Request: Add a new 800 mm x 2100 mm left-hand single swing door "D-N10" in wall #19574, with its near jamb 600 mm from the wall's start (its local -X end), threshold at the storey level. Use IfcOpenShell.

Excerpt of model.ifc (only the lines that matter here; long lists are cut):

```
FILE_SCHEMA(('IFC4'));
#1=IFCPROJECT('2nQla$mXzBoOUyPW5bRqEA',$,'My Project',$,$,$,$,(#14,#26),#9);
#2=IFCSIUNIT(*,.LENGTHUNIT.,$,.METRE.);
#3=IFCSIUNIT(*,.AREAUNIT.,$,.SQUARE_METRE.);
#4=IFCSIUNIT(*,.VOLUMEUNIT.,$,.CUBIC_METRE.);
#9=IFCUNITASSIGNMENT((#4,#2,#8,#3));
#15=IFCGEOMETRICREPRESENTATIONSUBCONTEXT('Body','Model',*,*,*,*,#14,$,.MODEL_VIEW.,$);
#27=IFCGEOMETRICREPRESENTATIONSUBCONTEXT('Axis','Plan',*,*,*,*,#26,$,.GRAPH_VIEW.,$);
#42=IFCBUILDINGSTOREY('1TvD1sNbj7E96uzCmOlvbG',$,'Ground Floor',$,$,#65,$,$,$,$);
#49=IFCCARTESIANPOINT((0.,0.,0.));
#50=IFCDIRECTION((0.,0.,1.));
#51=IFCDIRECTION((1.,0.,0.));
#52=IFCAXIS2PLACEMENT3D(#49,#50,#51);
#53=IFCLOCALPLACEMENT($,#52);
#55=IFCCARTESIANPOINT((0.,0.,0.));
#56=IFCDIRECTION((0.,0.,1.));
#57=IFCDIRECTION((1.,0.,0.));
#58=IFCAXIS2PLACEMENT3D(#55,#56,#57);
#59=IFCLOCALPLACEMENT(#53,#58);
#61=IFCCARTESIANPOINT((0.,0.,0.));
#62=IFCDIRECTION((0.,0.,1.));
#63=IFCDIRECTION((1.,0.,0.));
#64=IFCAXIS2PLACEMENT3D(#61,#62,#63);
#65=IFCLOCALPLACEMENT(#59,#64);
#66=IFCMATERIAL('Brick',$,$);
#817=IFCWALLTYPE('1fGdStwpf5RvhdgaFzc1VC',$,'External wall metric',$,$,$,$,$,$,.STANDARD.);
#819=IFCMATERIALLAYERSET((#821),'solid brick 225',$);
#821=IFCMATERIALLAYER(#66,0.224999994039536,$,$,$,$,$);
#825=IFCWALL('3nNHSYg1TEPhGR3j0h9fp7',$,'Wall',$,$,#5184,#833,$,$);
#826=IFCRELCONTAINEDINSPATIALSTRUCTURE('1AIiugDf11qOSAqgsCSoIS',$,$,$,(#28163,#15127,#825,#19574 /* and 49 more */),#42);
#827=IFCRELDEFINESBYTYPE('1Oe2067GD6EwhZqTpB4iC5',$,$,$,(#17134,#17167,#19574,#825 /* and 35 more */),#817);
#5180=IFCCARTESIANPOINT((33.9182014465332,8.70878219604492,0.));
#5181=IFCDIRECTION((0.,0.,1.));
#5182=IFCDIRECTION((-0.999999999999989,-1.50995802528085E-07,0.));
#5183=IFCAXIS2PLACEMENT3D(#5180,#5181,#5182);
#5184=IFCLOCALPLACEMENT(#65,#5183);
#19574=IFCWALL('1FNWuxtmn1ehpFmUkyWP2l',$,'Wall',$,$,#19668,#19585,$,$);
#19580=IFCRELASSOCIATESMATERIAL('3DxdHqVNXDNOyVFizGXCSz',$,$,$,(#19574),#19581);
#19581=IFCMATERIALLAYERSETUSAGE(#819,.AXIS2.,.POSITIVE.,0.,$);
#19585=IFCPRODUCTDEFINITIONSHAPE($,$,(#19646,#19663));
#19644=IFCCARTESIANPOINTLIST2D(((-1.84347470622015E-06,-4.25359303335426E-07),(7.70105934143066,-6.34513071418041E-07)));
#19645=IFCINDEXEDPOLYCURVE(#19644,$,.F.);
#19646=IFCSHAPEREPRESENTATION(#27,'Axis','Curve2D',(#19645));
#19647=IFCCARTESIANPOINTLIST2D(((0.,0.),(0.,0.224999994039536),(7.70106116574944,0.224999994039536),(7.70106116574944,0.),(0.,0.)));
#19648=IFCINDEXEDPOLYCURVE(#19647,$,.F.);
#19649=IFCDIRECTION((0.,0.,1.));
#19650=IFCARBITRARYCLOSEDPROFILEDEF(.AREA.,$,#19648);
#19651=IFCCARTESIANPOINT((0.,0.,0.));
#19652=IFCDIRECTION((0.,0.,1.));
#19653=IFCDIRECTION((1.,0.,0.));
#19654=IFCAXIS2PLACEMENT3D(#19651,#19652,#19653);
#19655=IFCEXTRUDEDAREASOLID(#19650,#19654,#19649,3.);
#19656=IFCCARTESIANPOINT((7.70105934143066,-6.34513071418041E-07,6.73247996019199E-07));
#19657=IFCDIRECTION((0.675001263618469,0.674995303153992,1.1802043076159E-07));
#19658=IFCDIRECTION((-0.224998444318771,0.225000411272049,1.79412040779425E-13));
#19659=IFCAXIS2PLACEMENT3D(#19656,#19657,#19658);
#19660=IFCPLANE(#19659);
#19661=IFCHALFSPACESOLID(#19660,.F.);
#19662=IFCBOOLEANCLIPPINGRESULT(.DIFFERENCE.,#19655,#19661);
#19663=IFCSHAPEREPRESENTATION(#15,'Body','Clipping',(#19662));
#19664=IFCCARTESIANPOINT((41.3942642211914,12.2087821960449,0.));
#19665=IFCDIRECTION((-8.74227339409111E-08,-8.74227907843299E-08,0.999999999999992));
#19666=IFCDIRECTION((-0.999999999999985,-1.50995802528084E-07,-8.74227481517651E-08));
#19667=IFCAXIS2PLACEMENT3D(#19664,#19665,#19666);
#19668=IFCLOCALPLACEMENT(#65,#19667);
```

```python
import numpy as np
import ifcopenshell
import ifcopenshell.api.feature
import ifcopenshell.api.geometry
import ifcopenshell.api.root
import ifcopenshell.api.spatial
import ifcopenshell.geom
import ifcopenshell.util.element
import ifcopenshell.util.placement
import ifcopenshell.util.representation
import ifcopenshell.util.shape
import ifcopenshell.util.unit

model = ifcopenshell.open("model.ifc")
unit_scale = ifcopenshell.util.unit.calculate_unit_scale(model)
settings = ifcopenshell.geom.settings()


def volume(element):
    """Net volume in cubic metres, openings subtracted."""
    shape = ifcopenshell.geom.create_shape(settings, element)
    return ifcopenshell.util.shape.get_volume(shape.geometry)


wall = model.by_id(19574)
storey = ifcopenshell.util.element.get_container(wall, ifc_class="IfcBuildingStorey")
context = ifcopenshell.util.representation.get_context(model, "Model", "Body", "MODEL_VIEW")
before = volume(wall)

width, height, from_end, sill = 0.8, 2.1, 0.6, 0.0  # metres

# The wall runs along its own X axis, and the end named is its -X end.
wall_shape = ifcopenshell.geom.create_shape(settings, wall)
x, y, z = ifcopenshell.util.shape.get_vertices(wall_shape.geometry).T
start = x.min() + from_end
face, thickness = float(y.min()), float(y.max() - y.min())
wall_matrix = ifcopenshell.util.placement.get_local_placement(wall.ObjectPlacement)
level = ifcopenshell.util.placement.get_local_placement(storey.ObjectPlacement)[2, 3]


def in_wall(x, y):
    """Placement at x, y metres in the wall's axes, at sill height."""
    matrix = wall_matrix.copy()
    matrix[:, 3] = wall_matrix @ np.array([x / unit_scale, y / unit_scale, 0.0, 1.0])
    matrix[2, 3] = level + sill / unit_scale
    return matrix


# Opening: a box that overshoots both wall faces by 50 mm.
opening = ifcopenshell.api.root.create_entity(model, ifc_class="IfcOpeningElement", predefined_type="OPENING")
box = ifcopenshell.api.geometry.add_wall_representation(
    model, context=context, length=width, height=height, thickness=thickness + 0.1
)
ifcopenshell.api.geometry.assign_representation(model, product=opening, representation=box)
ifcopenshell.api.geometry.edit_object_placement(model, product=opening, matrix=in_wall(start, face - 0.05), is_si=False)
ifcopenshell.api.feature.add_feature(model, feature=opening, element=wall)

door = ifcopenshell.api.root.create_entity(model, ifc_class="IfcDoor", name="D-N10", predefined_type="DOOR")
door.OverallWidth, door.OverallHeight = width / unit_scale, height / unit_scale
door.OperationType = "SINGLE_SWING_LEFT"
body = ifcopenshell.api.geometry.add_door_representation(
    model,
    context=context,
    overall_width=door.OverallWidth,
    overall_height=door.OverallHeight,
    operation_type="SINGLE_SWING_LEFT",
    lining_properties={"LiningDepth": thickness / unit_scale, "ThresholdDepth": thickness / unit_scale},
)
ifcopenshell.api.geometry.assign_representation(model, product=door, representation=body)
ifcopenshell.api.spatial.assign_container(model, products=[door], relating_structure=storey)
ifcopenshell.api.feature.add_filling(model, opening=opening, element=door)

# The lining spans the wall, so the door starts at the wall face.
ifcopenshell.api.geometry.edit_object_placement(model, product=door, matrix=in_wall(start, face), is_si=False)

after = volume(wall)

print(f"wall volume {before:.3f} -> {after:.3f} m3")

model.write("model_rev.ifc")
```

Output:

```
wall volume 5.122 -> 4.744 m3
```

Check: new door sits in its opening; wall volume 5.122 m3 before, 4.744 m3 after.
